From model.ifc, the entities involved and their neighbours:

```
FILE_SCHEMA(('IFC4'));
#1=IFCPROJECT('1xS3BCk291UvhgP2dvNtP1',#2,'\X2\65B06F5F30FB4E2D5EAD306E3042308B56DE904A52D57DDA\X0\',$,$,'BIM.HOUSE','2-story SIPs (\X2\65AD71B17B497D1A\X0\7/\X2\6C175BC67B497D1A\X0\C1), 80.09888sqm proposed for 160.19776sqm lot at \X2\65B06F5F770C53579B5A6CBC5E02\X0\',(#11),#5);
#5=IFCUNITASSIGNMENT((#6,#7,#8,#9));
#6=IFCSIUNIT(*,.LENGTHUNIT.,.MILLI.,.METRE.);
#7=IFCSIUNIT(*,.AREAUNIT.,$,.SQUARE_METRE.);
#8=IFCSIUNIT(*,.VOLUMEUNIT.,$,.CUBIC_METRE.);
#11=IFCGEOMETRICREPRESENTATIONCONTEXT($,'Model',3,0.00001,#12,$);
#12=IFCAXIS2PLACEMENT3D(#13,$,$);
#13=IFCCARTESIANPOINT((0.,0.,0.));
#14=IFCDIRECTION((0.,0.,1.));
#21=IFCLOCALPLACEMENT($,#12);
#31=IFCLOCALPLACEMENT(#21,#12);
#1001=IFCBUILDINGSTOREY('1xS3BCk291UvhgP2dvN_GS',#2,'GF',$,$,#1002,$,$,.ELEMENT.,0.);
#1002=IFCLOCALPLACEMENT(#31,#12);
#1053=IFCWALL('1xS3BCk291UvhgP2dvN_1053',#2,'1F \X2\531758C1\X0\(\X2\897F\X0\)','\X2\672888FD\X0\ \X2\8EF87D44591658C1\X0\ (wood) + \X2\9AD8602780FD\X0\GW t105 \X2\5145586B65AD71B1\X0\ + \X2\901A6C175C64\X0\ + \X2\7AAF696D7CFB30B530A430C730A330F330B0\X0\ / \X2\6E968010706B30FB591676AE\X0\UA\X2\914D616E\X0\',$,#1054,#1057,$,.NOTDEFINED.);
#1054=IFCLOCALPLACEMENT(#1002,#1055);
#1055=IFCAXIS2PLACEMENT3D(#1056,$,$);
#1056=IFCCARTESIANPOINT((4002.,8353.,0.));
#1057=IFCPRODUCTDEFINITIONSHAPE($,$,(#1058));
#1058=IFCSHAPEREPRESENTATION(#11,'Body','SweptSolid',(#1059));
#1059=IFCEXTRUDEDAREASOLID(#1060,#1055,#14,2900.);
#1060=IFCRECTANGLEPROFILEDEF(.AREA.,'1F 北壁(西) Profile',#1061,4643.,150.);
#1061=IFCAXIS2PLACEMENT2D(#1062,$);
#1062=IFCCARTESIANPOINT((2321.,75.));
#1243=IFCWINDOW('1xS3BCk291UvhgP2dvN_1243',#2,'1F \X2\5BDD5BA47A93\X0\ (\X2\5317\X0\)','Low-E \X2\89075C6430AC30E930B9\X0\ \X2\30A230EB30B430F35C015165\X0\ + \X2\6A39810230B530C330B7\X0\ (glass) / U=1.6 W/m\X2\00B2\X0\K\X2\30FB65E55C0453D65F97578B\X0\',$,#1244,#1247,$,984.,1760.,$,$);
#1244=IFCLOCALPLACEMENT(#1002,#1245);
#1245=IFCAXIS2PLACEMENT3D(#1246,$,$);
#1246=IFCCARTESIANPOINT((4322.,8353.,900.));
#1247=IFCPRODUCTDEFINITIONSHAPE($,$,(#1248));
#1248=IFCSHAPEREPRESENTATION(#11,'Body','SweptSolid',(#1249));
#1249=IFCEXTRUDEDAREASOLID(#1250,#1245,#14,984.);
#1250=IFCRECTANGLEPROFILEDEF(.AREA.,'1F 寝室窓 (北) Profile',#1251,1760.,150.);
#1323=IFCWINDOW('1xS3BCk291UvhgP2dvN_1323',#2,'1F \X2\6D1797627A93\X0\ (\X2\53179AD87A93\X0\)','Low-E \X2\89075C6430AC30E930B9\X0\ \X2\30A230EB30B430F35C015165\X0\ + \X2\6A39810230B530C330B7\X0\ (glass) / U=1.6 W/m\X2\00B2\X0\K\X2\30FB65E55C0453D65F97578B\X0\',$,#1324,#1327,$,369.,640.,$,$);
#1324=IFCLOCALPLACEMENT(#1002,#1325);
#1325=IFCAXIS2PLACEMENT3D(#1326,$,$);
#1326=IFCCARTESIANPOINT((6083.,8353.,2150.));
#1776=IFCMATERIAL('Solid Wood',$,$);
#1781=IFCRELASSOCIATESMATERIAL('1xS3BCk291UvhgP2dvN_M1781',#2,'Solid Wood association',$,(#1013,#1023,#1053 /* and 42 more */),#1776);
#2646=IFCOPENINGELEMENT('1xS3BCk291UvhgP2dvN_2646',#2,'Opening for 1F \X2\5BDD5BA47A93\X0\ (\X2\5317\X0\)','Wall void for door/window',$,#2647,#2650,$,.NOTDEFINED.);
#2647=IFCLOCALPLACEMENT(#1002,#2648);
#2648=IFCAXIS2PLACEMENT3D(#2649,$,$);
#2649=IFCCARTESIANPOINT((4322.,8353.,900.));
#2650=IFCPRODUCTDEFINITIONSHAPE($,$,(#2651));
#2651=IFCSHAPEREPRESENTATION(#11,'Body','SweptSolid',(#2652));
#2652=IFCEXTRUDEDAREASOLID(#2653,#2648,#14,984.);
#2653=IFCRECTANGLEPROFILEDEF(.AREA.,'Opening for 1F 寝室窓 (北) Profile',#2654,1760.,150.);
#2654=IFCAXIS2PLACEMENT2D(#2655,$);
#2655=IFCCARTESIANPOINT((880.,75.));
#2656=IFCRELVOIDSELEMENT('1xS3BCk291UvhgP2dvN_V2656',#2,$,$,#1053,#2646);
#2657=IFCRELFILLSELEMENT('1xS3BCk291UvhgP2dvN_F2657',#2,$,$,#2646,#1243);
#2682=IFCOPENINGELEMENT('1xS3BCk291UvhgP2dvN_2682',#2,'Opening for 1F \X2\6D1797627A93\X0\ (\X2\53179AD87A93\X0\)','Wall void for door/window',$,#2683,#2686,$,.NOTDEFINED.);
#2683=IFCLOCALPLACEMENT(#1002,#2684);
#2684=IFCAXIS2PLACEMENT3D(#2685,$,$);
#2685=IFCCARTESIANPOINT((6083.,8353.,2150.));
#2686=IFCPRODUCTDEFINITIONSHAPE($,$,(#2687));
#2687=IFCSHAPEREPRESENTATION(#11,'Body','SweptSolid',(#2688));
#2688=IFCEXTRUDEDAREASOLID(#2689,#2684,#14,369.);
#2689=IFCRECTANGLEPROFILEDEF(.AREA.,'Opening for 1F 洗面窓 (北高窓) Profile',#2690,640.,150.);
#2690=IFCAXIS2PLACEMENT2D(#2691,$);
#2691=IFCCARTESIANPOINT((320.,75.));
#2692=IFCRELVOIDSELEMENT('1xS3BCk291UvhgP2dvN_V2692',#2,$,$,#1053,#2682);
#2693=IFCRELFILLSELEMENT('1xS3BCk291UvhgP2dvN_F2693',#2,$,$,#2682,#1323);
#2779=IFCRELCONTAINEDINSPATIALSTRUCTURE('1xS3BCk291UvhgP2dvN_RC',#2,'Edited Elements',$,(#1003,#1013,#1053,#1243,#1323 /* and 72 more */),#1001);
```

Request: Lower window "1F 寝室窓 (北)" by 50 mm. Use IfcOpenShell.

```python
import numpy as np
import ifcopenshell
import ifcopenshell.api.geometry
import ifcopenshell.util.placement
import ifcopenshell.util.unit

model = ifcopenshell.open("model.ifc")
unit_scale = ifcopenshell.util.unit.calculate_unit_scale(model)

window = model.by_guid("1xS3BCk291UvhgP2dvN_1243")
opening = window.FillsVoids[0].RelatingOpeningElement
dz = -0.05 / unit_scale

shift = np.array([0.0, 0.0, dz])
# The window is not placed relative to its opening, so move both.
for product in (opening, window):
    matrix = ifcopenshell.util.placement.get_local_placement(product.ObjectPlacement)
    matrix[:3, 3] += shift
    ifcopenshell.api.geometry.edit_object_placement(model, product=product, matrix=matrix, is_si=False)

print(f"moved by {dz * unit_scale:+.3f} m")

model.write("model_v2.ifc")
```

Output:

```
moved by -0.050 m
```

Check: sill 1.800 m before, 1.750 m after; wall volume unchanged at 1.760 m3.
